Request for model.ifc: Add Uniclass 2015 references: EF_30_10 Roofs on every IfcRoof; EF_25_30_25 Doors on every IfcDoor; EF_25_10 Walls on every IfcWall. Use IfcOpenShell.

First a look at what the model holds.

```python
import ifcopenshell

model = ifcopenshell.open("model.ifc")
print(model.schema)
print("classifications:", [c.Name for c in model.by_type("IfcClassification")])
for ifc_class in ("IfcDoor", "IfcRoof", "IfcStair", "IfcWall", "IfcWindow"):
    print(ifc_class, len(model.by_type(ifc_class)))
```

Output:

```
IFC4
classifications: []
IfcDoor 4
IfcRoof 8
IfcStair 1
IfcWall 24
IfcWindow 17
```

```python
import ifcopenshell
import ifcopenshell.api.classification

model = ifcopenshell.open("model.ifc")

system = ifcopenshell.api.classification.add_classification(model, classification="Uniclass 2015")

codes = {
    "IfcRoof": ("EF_30_10", "Roofs"),
    "IfcDoor": ("EF_25_30_25", "Doors"),
    "IfcWall": ("EF_25_10", "Walls"),
}
for ifc_class, (code, name) in codes.items():
    products = model.by_type(ifc_class)
    ifcopenshell.api.classification.add_reference(
        model, products=products, classification=system, identification=code, name=name
    )
    print(code, len(products))

model.write("model_rev.ifc")
```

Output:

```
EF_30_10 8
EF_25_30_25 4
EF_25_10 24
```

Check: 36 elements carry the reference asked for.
